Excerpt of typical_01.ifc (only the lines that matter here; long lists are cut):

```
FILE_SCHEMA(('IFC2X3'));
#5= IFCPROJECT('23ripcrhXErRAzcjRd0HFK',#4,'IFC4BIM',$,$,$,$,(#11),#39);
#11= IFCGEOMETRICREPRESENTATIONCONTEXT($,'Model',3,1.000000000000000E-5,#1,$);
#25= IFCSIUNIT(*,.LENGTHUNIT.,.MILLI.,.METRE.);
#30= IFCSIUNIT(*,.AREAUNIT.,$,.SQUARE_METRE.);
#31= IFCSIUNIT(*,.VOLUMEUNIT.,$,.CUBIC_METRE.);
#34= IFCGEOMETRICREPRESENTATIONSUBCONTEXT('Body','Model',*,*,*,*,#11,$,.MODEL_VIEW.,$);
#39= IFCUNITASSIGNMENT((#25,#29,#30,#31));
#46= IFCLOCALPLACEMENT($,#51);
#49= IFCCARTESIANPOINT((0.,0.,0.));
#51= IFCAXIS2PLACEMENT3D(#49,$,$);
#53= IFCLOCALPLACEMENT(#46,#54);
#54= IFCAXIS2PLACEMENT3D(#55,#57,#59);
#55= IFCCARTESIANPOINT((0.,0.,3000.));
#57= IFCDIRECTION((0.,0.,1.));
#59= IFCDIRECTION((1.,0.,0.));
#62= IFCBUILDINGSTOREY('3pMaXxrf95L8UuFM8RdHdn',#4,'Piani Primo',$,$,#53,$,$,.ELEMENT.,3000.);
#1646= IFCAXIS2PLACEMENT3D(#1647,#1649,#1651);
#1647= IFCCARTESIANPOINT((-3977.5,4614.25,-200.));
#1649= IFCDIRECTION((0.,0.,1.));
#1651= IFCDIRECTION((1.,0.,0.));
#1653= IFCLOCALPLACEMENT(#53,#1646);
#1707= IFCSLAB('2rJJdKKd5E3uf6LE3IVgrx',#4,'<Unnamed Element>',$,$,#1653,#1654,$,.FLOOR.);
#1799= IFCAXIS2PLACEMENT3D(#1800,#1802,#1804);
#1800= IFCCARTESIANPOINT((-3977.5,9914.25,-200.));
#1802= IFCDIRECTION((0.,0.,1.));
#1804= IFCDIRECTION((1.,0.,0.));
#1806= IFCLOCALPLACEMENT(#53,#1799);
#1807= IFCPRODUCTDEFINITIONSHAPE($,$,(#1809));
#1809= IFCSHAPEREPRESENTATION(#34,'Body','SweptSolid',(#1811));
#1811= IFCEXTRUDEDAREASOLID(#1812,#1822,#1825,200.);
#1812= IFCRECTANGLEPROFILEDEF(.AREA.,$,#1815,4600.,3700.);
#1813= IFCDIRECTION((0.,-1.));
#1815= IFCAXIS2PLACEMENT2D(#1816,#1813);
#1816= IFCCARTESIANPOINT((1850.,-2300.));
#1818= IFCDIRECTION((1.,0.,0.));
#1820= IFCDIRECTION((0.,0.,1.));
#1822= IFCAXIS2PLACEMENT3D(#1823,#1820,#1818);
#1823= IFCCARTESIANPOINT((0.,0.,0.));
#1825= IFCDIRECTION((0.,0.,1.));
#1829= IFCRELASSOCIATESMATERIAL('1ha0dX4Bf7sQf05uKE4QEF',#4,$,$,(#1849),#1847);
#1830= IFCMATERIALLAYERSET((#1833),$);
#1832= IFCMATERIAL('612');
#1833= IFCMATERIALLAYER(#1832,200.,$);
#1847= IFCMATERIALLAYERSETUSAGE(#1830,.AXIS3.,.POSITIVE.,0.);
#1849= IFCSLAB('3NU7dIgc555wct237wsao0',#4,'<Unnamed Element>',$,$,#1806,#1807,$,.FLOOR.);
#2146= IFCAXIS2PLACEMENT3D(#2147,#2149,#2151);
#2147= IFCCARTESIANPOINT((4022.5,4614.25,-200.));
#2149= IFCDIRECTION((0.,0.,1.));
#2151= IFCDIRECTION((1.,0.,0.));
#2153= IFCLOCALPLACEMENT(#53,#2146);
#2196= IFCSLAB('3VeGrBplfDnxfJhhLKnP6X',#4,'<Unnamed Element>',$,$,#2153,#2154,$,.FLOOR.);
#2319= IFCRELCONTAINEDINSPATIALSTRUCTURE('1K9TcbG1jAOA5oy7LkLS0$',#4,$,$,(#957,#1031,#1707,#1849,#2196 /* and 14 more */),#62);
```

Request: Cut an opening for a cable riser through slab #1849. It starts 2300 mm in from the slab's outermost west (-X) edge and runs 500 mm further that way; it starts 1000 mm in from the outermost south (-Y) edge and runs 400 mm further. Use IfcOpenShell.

```python
import numpy as np
import ifcopenshell
import ifcopenshell.api.feature
import ifcopenshell.api.geometry
import ifcopenshell.api.root
import ifcopenshell.geom
import ifcopenshell.util.placement
import ifcopenshell.util.representation
import ifcopenshell.util.shape
import ifcopenshell.util.unit

model = ifcopenshell.open("typical_01.ifc")
unit_scale = ifcopenshell.util.unit.calculate_unit_scale(model)
settings = ifcopenshell.geom.settings()


def volume(element):
    """Net volume in cubic metres, openings subtracted."""
    shape = ifcopenshell.geom.create_shape(settings, element)
    return ifcopenshell.util.shape.get_volume(shape.geometry)


slab = model.by_guid("3NU7dIgc555wct237wsao0")
before = volume(slab)

# Extent in the slab's own axes, in metres. The edges named are its -X and -Y sides.
slab_shape = ifcopenshell.geom.create_shape(settings, slab)
vertices = ifcopenshell.util.shape.get_vertices(slab_shape.geometry)
x_min, y_min, bottom = vertices.min(axis=0)
top = vertices[:, 2].max()

opening = ifcopenshell.api.root.create_entity(model, ifc_class="IfcOpeningElement", name="Cable riser opening")
context = ifcopenshell.util.representation.get_context(model, "Model", "Body", "MODEL_VIEW")
width, depth = 0.5, 0.4
outline = [(0.0, 0.0), (width, 0.0), (width, depth), (0.0, depth), (0.0, 0.0)]
# Overshoot both faces by 50 mm so the cut is clean.
shape = ifcopenshell.api.geometry.add_slab_representation(
    model, context=context, depth=top - bottom + 0.1, polyline=outline
)
ifcopenshell.api.geometry.assign_representation(model, product=opening, representation=shape)

matrix = ifcopenshell.util.placement.get_local_placement(slab.ObjectPlacement)
matrix[:, 3] = matrix @ np.append(np.array([x_min + 2.3, y_min + 1, bottom - 0.05]) / unit_scale, 1.0)
ifcopenshell.api.geometry.edit_object_placement(model, product=opening, matrix=matrix, is_si=False)
ifcopenshell.api.feature.add_feature(model, feature=opening, element=slab)

after = volume(slab)

print(f"slab volume {before:.3f} -> {after:.3f} m3")

model.write("typical_01_v2.ifc")
```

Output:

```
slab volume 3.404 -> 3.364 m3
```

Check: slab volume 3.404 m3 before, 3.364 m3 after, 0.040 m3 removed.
